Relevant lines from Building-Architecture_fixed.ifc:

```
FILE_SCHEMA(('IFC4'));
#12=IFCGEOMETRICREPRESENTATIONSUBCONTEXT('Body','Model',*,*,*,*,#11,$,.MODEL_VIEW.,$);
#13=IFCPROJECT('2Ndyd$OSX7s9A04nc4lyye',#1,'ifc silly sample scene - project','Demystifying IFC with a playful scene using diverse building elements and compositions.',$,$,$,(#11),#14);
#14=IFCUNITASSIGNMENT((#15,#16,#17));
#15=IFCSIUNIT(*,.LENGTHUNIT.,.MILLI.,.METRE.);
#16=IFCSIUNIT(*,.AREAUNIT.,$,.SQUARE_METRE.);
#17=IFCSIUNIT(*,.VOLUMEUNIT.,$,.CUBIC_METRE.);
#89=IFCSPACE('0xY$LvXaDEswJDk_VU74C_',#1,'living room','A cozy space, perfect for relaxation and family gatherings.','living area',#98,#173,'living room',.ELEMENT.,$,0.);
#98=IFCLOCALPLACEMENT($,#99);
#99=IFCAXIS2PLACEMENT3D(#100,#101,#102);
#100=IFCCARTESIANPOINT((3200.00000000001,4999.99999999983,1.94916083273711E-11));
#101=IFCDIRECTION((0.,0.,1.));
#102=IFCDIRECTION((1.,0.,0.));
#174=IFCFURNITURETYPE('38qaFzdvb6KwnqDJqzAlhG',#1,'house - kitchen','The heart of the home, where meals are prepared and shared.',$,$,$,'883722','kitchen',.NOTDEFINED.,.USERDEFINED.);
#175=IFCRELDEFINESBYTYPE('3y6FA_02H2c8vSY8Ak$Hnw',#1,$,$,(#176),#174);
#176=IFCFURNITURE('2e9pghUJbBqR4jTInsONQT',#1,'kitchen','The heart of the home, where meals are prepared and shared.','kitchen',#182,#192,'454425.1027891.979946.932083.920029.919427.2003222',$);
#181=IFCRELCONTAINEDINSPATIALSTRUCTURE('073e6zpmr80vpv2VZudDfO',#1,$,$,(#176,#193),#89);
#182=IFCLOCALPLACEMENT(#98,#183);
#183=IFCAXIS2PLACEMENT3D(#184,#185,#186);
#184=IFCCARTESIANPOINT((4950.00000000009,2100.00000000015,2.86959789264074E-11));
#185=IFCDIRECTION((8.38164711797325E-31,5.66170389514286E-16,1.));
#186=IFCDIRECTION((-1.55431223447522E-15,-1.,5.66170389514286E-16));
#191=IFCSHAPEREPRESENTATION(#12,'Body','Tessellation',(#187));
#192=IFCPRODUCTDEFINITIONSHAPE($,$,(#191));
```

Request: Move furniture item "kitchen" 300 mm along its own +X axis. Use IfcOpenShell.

```python
import ifcopenshell
import ifcopenshell.api.geometry
import ifcopenshell.util.placement
import ifcopenshell.util.unit

model = ifcopenshell.open("Building-Architecture_fixed.ifc")
unit_scale = ifcopenshell.util.unit.calculate_unit_scale(model)

item = model.by_guid("2e9pghUJbBqR4jTInsONQT")
matrix = ifcopenshell.util.placement.get_local_placement(item.ObjectPlacement)
matrix[:3, 3] += matrix[:3, 0] * 0.3 / unit_scale
ifcopenshell.api.geometry.edit_object_placement(model, product=item, matrix=matrix, is_si=False)

print(ifcopenshell.util.placement.get_local_placement(item.ObjectPlacement).round(3) + 0.0)

model.write("Building-Architecture_fixed_v2.ifc")
```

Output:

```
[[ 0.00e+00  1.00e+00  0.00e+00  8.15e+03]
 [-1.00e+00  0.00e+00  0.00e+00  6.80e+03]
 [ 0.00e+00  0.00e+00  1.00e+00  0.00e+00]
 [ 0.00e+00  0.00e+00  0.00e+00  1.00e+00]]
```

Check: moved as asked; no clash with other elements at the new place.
